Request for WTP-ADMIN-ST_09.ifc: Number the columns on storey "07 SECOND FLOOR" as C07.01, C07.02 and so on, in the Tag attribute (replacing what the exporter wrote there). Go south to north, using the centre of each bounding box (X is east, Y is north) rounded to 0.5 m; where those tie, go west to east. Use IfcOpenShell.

First a look at what the model holds.

```python
import ifcopenshell
import ifcopenshell.util.element
import ifcopenshell.util.placement

model = ifcopenshell.open("WTP-ADMIN-ST_09.ifc")
print(model.schema)
storey = next(s for s in model.by_type("IfcBuildingStorey") if s.Name == "07 SECOND FLOOR")
columns = [e for e in ifcopenshell.util.element.get_decomposition(storey) if e.is_a("IfcColumn")]
for e in sorted(columns, key=lambda e: e.id()):
    origin = ifcopenshell.util.placement.get_local_placement(e.ObjectPlacement)[:3, 3]
    print(e.id(), e.Tag, e.Name, origin.round(2) + 0.0, sep=" | ")
```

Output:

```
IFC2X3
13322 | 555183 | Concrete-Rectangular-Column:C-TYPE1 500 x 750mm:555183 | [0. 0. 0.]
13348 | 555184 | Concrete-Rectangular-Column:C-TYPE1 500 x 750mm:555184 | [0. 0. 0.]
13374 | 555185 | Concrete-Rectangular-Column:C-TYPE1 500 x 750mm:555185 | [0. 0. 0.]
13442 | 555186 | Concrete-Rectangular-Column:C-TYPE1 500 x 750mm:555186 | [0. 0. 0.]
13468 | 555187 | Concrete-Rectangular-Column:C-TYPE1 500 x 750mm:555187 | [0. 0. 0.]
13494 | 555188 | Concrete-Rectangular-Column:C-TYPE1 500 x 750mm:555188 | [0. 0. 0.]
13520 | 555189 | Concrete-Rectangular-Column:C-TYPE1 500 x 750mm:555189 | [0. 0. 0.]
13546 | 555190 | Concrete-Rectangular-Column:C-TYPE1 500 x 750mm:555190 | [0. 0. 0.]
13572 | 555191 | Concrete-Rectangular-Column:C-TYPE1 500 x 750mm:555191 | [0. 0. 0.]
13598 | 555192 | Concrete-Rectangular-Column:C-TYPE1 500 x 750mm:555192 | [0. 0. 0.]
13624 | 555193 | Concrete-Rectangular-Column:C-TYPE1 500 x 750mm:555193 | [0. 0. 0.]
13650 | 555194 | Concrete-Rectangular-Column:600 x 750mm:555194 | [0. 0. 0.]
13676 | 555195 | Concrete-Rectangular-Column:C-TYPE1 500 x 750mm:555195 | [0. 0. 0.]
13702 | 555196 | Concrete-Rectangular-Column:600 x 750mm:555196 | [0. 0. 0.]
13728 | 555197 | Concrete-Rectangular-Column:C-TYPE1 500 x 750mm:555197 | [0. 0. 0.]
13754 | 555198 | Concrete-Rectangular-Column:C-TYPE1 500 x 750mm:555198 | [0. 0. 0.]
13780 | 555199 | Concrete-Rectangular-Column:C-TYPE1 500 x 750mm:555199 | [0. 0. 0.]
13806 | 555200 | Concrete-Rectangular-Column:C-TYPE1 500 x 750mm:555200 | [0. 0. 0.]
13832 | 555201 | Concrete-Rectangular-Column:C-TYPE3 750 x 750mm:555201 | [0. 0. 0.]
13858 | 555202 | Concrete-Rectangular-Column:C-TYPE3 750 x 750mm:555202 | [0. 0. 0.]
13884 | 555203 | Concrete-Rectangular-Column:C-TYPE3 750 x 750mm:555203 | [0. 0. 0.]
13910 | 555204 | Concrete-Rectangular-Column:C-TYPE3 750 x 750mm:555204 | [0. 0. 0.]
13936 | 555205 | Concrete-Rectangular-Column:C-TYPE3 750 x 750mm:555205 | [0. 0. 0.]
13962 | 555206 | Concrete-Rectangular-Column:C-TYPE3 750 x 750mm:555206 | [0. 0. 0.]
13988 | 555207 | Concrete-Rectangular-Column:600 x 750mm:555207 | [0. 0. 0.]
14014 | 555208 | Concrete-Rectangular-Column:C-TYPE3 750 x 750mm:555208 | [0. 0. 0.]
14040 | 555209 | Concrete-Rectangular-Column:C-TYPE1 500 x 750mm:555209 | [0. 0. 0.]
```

```python
import ifcopenshell
import ifcopenshell.geom
import ifcopenshell.util.element
import ifcopenshell.util.shape

model = ifcopenshell.open("WTP-ADMIN-ST_09.ifc")
settings = ifcopenshell.geom.settings()
settings.set("use-world-coords", True)


def centre(element):
    shape = ifcopenshell.geom.create_shape(settings, element)
    return ifcopenshell.util.shape.get_bbox_centroid(shape.geometry)


storey = next(s for s in model.by_type("IfcBuildingStorey") if s.Name == "07 SECOND FLOOR")
columns = [e for e in ifcopenshell.util.element.get_decomposition(storey) if e.is_a("IfcColumn")]

# Insertion points can sit at a corner or the storey origin, so sort by the geometry (in metres).
centres = {e: centre(e) for e in columns}
columns.sort(key=lambda e: (round(centres[e][1] / 0.5), centres[e][0]))

for i, e in enumerate(columns, start=1):
    number = f"C07.{i:02d}"
    e.Tag = number
    print(e.id(), number)

model.write("WTP-ADMIN-ST_09_rev.ifc")
```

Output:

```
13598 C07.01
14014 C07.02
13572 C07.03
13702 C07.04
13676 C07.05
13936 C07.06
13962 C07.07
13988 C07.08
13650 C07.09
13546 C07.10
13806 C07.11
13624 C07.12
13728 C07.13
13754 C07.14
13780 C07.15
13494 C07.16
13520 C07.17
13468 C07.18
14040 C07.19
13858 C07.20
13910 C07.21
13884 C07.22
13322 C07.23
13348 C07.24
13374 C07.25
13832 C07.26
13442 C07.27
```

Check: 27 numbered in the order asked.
